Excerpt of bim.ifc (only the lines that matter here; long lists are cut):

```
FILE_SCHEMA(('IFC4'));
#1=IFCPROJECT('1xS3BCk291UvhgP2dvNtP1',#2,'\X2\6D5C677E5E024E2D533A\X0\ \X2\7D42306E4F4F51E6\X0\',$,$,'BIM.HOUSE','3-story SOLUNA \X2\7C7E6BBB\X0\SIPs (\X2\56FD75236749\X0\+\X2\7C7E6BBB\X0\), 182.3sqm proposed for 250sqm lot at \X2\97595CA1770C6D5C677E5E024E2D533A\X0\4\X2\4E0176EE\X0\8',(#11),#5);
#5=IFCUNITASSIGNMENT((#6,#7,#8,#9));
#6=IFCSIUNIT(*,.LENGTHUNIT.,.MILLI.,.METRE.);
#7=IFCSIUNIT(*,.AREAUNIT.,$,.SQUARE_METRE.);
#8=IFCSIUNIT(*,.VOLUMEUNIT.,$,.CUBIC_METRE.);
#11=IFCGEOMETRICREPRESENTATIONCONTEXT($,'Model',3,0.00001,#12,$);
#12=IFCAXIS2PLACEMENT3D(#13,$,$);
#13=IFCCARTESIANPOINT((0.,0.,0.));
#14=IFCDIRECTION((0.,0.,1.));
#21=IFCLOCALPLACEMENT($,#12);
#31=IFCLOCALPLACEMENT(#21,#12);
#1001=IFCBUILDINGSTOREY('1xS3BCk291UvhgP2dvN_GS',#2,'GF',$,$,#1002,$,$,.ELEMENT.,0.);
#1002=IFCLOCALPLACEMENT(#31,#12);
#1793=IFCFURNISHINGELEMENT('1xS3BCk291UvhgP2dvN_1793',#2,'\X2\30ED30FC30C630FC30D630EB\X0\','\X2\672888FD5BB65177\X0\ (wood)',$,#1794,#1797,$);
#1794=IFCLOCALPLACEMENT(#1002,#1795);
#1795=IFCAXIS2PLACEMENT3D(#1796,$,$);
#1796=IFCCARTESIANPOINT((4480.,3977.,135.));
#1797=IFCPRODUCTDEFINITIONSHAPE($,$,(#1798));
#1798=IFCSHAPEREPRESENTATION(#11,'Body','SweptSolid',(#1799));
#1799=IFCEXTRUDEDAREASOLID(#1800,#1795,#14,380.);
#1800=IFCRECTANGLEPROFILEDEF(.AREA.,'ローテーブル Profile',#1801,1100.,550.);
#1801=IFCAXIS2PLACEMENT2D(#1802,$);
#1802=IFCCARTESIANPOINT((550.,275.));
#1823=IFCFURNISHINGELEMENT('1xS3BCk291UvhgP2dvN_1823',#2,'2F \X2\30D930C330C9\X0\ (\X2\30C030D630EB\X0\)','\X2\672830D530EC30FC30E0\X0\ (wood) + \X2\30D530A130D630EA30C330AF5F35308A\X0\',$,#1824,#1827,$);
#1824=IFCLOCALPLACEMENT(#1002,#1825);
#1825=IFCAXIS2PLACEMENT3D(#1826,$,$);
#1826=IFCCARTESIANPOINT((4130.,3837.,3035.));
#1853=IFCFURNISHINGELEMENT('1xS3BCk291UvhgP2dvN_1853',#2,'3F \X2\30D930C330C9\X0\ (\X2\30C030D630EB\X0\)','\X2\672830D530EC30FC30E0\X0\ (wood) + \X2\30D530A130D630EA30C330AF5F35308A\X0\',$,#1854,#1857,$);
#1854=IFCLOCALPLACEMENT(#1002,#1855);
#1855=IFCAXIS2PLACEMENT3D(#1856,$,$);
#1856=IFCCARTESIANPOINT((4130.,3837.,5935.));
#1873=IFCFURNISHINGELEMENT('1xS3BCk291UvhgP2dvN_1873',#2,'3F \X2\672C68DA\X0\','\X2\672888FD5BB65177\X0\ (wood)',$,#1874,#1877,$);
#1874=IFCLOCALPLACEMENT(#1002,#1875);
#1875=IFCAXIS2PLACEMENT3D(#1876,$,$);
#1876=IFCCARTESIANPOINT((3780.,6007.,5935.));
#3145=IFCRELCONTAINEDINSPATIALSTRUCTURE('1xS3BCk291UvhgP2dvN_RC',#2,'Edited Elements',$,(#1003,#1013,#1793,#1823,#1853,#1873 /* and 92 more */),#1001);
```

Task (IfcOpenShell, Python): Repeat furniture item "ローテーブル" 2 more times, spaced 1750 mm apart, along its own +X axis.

```python
import ifcopenshell
import ifcopenshell.api.geometry
import ifcopenshell.api.root
import ifcopenshell.util.element
import ifcopenshell.util.placement
import ifcopenshell.util.unit

model = ifcopenshell.open("bim.ifc")
unit_scale = ifcopenshell.util.unit.calculate_unit_scale(model)


def reuse_history(source, copy):
    """copy_class also copies each property set's owner history, people and application; keep the originals."""
    for rel in copy.IsDefinedBy:
        if rel.is_a("IfcRelDefinesByProperties") and (history := rel.RelatingPropertyDefinition.OwnerHistory):
            rel.RelatingPropertyDefinition.OwnerHistory = source.OwnerHistory
            ifcopenshell.util.element.remove_deep2(model, history)


source = model.by_id(1793)
base = ifcopenshell.util.placement.get_local_placement(source.ObjectPlacement)
step = base[:3, 0] * 1.75 / unit_scale

for i in range(1, 3):
    copy = ifcopenshell.api.root.copy_class(model, product=source)
    copy.Representation = ifcopenshell.util.element.copy_deep(
        model, source.Representation, exclude=["IfcGeometricRepresentationContext", "IfcRepresentationMap"]
    )
    reuse_history(source, copy)
    matrix = base.copy()
    matrix[:3, 3] += i * step
    print("added at", matrix[:3, 3].round(3) + 0.0)
    ifcopenshell.api.geometry.edit_object_placement(model, product=copy, matrix=matrix, is_si=False)

model.write("bim_rev.ifc")
```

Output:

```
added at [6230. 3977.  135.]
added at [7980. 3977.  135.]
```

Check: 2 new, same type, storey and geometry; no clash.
